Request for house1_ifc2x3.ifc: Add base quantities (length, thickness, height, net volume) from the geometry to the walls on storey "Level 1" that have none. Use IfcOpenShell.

First a look at what the model holds.

```python
import ifcopenshell
import ifcopenshell.util.element
import ifcopenshell.util.unit

model = ifcopenshell.open("house1_ifc2x3.ifc")
print(model.schema)
for unit_type in ("LENGTHUNIT", "AREAUNIT", "VOLUMEUNIT"):
    print(unit_type, ifcopenshell.util.unit.calculate_unit_scale(model, unit_type))
storey = next(s for s in model.by_type("IfcBuildingStorey") if s.Name == "Level 1")
walls = [e for e in ifcopenshell.util.element.get_decomposition(storey) if e.is_a("IfcWall")]
for e in sorted(walls, key=lambda e: e.id()):
    print(e.id(), e.is_a(), e.Name, list(ifcopenshell.util.element.get_psets(e, qtos_only=True)), sep=" | ")
```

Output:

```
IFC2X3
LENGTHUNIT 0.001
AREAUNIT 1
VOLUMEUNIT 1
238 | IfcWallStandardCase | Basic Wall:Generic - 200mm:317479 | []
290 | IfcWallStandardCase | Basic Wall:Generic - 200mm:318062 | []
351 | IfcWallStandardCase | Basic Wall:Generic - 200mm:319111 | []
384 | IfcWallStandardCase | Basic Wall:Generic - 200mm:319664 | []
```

```python
import ifcopenshell
import ifcopenshell.api.pset
import ifcopenshell.geom
import ifcopenshell.util.element
import ifcopenshell.util.shape
import ifcopenshell.util.unit

model = ifcopenshell.open("house1_ifc2x3.ifc")
unit_scale = ifcopenshell.util.unit.calculate_unit_scale(model)
volume_scale = ifcopenshell.util.unit.calculate_unit_scale(model, "VOLUMEUNIT")
settings = ifcopenshell.geom.settings()

storey = next(s for s in model.by_type("IfcBuildingStorey") if s.Name == "Level 1")
walls = [e for e in ifcopenshell.util.element.get_decomposition(storey) if e.is_a("IfcWall")]

for e in sorted(walls, key=lambda e: e.id()):
    if ifcopenshell.util.element.get_psets(e, qtos_only=True, should_inherit=False):
        continue
    # Geometry comes back in metres, in the element's own axes.
    shape = ifcopenshell.geom.create_shape(settings, e)
    values = {
        "Length": ifcopenshell.util.shape.get_x(shape.geometry) / unit_scale,
        "Width": ifcopenshell.util.shape.get_y(shape.geometry) / unit_scale,
        "Height": ifcopenshell.util.shape.get_z(shape.geometry) / unit_scale,
        "NetVolume": ifcopenshell.util.shape.get_volume(shape.geometry) / volume_scale,
    }
    qto = ifcopenshell.api.pset.add_qto(model, product=e, name="BaseQuantities")
    ifcopenshell.api.pset.edit_qto(model, qto=qto, properties=values)
    print(e.id(), {k: round(v, 3) for k, v in values.items()})

model.write("house1_ifc2x3_updated.ifc")
```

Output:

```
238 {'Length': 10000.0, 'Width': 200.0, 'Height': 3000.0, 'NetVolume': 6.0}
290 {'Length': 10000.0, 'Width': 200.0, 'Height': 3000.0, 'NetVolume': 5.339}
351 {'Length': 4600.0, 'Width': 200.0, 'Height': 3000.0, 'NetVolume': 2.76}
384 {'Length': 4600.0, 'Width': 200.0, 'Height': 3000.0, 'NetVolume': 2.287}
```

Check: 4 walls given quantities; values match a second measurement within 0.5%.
